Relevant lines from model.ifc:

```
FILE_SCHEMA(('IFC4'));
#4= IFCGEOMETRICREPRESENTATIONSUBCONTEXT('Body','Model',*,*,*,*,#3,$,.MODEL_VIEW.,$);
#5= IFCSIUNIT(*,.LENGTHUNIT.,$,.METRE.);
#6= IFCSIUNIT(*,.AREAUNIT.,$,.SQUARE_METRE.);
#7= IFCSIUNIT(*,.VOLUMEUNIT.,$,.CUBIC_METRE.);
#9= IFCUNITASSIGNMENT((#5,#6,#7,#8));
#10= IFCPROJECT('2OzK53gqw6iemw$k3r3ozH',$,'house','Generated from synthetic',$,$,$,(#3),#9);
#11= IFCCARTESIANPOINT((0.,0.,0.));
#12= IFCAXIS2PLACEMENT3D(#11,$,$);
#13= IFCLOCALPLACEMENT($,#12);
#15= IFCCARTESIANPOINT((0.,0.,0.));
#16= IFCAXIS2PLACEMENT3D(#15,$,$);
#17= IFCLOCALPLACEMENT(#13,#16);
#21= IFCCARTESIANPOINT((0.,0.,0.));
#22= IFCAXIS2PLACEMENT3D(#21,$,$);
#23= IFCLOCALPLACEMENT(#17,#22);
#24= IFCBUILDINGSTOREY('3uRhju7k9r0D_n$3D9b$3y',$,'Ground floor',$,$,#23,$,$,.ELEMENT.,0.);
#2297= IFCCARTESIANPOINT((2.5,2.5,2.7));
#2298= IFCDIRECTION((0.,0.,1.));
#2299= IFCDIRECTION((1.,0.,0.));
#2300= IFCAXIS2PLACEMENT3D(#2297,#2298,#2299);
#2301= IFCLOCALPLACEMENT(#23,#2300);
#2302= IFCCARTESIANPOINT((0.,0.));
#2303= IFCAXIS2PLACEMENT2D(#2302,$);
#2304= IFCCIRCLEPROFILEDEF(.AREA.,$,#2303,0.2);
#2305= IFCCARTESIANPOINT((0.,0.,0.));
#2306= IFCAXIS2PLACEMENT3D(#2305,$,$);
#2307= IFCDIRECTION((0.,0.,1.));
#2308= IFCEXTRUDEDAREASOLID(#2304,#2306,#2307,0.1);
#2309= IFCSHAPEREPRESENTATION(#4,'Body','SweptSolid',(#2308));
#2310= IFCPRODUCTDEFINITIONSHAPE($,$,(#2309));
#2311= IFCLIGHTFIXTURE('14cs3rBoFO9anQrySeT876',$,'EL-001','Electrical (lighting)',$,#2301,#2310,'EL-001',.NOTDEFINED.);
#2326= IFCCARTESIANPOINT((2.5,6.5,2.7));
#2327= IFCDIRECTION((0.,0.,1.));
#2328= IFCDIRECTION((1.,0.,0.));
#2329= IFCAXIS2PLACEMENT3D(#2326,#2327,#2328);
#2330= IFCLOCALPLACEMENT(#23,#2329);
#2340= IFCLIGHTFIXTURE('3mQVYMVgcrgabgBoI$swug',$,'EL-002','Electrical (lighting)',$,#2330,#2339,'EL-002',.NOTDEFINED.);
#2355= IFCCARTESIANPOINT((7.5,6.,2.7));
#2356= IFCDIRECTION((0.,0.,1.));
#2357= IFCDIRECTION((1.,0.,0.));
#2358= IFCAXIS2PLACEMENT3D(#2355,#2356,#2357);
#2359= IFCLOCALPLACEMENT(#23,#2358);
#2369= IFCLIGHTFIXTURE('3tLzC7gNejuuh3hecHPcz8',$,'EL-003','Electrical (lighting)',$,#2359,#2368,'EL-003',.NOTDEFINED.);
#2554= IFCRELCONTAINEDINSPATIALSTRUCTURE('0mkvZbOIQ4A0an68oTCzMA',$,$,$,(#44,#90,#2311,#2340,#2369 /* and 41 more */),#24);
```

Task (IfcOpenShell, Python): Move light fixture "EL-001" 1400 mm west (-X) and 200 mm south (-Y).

```python
import ifcopenshell
import ifcopenshell.api.geometry
import ifcopenshell.util.placement

model = ifcopenshell.open("model.ifc")

item = model.by_guid("14cs3rBoFO9anQrySeT876")
matrix = ifcopenshell.util.placement.get_local_placement(item.ObjectPlacement)
matrix[0, 3] -= 1.4
matrix[1, 3] -= 0.2
ifcopenshell.api.geometry.edit_object_placement(model, product=item, matrix=matrix, is_si=False)

print(ifcopenshell.util.placement.get_local_placement(item.ObjectPlacement).round(3) + 0.0)

model.write("model_v2.ifc")
```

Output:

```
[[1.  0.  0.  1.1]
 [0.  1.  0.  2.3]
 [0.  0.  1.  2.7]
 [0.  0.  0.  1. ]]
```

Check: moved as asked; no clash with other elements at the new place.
